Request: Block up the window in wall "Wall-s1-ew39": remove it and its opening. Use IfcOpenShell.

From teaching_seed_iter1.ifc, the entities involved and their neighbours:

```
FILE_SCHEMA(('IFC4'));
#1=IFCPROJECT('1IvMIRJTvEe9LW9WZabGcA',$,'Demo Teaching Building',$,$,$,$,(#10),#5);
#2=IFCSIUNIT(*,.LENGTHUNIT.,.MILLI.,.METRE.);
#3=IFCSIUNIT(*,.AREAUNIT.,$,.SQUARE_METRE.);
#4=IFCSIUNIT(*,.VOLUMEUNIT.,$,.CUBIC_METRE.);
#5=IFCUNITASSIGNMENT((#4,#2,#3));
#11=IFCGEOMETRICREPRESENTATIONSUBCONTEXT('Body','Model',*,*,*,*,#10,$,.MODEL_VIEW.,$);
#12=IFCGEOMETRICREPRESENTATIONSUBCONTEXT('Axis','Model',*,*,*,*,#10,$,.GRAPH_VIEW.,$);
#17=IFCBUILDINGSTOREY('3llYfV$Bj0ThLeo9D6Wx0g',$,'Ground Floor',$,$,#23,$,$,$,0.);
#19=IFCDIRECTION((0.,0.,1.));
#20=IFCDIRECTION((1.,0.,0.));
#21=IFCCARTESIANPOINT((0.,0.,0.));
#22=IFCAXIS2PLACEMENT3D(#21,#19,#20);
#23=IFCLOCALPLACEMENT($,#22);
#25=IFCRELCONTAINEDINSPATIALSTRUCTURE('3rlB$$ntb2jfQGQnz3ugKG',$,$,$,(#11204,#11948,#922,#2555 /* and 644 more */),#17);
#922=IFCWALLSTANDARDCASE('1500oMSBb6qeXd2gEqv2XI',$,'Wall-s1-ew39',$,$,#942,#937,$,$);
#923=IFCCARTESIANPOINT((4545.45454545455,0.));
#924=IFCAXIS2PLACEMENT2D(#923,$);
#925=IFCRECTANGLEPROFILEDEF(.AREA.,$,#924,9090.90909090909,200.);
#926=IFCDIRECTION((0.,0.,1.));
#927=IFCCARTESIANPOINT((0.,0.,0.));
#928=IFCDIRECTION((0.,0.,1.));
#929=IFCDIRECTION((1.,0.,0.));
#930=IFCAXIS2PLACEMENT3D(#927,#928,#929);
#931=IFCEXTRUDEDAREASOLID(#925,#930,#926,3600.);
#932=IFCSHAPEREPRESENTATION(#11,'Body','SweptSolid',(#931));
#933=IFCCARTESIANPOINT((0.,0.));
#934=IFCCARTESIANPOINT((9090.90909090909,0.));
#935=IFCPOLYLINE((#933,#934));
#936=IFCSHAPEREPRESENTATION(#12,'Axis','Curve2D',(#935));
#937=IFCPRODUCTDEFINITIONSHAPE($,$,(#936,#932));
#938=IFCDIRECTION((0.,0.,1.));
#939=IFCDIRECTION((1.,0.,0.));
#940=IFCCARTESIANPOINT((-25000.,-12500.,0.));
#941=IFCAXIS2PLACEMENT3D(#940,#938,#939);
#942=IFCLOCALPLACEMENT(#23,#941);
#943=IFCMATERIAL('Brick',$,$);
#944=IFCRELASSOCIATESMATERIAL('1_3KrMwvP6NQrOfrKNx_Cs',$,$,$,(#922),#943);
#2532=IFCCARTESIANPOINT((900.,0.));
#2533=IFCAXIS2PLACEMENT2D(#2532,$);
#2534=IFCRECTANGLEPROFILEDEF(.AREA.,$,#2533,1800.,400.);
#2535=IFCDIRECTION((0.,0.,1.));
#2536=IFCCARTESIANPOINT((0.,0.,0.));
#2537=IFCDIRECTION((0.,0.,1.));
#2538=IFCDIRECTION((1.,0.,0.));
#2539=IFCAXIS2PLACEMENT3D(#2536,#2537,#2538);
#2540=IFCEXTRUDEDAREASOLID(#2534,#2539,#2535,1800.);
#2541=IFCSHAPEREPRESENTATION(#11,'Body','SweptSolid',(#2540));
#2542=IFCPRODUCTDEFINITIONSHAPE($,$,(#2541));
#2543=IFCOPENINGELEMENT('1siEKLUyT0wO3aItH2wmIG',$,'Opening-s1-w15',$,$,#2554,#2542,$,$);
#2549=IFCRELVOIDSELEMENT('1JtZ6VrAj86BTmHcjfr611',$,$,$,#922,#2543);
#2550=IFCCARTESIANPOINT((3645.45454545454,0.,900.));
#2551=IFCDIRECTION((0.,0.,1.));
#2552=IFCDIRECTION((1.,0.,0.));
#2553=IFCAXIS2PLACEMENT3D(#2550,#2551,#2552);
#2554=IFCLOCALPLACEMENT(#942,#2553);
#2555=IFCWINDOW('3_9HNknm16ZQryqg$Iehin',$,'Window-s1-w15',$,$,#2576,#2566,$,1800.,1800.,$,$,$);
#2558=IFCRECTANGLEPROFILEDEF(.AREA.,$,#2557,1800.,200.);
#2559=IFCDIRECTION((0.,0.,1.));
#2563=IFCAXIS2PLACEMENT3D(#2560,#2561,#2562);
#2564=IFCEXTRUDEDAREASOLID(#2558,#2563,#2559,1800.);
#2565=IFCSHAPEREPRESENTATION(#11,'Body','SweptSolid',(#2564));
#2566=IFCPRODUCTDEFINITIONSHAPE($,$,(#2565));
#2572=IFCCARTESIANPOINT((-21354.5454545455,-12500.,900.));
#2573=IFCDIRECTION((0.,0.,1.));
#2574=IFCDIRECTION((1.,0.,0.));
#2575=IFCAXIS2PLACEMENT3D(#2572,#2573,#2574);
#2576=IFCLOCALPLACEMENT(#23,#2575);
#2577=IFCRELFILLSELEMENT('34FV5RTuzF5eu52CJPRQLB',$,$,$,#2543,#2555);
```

```python
import ifcopenshell
import ifcopenshell.api.feature
import ifcopenshell.api.root
import ifcopenshell.geom
import ifcopenshell.util.shape

model = ifcopenshell.open("teaching_seed_iter1.ifc")
settings = ifcopenshell.geom.settings()


def volume(element):
    """Net volume in cubic metres, openings subtracted."""
    shape = ifcopenshell.geom.create_shape(settings, element)
    return ifcopenshell.util.shape.get_volume(shape.geometry)


window = model.by_guid("3_9HNknm16ZQryqg$Iehin")
opening = window.FillsVoids[0].RelatingOpeningElement
wall = opening.VoidsElements[0].RelatingBuildingElement
before = volume(wall)

ifcopenshell.api.root.remove_product(model, product=window)
ifcopenshell.api.feature.remove_feature(model, feature=opening)

after = volume(wall)

print(f"wall volume {before:.3f} -> {after:.3f} m3")

model.write("teaching_seed_iter1_edited.ifc")
```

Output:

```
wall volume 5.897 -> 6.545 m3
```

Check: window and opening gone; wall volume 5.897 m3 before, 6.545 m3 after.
